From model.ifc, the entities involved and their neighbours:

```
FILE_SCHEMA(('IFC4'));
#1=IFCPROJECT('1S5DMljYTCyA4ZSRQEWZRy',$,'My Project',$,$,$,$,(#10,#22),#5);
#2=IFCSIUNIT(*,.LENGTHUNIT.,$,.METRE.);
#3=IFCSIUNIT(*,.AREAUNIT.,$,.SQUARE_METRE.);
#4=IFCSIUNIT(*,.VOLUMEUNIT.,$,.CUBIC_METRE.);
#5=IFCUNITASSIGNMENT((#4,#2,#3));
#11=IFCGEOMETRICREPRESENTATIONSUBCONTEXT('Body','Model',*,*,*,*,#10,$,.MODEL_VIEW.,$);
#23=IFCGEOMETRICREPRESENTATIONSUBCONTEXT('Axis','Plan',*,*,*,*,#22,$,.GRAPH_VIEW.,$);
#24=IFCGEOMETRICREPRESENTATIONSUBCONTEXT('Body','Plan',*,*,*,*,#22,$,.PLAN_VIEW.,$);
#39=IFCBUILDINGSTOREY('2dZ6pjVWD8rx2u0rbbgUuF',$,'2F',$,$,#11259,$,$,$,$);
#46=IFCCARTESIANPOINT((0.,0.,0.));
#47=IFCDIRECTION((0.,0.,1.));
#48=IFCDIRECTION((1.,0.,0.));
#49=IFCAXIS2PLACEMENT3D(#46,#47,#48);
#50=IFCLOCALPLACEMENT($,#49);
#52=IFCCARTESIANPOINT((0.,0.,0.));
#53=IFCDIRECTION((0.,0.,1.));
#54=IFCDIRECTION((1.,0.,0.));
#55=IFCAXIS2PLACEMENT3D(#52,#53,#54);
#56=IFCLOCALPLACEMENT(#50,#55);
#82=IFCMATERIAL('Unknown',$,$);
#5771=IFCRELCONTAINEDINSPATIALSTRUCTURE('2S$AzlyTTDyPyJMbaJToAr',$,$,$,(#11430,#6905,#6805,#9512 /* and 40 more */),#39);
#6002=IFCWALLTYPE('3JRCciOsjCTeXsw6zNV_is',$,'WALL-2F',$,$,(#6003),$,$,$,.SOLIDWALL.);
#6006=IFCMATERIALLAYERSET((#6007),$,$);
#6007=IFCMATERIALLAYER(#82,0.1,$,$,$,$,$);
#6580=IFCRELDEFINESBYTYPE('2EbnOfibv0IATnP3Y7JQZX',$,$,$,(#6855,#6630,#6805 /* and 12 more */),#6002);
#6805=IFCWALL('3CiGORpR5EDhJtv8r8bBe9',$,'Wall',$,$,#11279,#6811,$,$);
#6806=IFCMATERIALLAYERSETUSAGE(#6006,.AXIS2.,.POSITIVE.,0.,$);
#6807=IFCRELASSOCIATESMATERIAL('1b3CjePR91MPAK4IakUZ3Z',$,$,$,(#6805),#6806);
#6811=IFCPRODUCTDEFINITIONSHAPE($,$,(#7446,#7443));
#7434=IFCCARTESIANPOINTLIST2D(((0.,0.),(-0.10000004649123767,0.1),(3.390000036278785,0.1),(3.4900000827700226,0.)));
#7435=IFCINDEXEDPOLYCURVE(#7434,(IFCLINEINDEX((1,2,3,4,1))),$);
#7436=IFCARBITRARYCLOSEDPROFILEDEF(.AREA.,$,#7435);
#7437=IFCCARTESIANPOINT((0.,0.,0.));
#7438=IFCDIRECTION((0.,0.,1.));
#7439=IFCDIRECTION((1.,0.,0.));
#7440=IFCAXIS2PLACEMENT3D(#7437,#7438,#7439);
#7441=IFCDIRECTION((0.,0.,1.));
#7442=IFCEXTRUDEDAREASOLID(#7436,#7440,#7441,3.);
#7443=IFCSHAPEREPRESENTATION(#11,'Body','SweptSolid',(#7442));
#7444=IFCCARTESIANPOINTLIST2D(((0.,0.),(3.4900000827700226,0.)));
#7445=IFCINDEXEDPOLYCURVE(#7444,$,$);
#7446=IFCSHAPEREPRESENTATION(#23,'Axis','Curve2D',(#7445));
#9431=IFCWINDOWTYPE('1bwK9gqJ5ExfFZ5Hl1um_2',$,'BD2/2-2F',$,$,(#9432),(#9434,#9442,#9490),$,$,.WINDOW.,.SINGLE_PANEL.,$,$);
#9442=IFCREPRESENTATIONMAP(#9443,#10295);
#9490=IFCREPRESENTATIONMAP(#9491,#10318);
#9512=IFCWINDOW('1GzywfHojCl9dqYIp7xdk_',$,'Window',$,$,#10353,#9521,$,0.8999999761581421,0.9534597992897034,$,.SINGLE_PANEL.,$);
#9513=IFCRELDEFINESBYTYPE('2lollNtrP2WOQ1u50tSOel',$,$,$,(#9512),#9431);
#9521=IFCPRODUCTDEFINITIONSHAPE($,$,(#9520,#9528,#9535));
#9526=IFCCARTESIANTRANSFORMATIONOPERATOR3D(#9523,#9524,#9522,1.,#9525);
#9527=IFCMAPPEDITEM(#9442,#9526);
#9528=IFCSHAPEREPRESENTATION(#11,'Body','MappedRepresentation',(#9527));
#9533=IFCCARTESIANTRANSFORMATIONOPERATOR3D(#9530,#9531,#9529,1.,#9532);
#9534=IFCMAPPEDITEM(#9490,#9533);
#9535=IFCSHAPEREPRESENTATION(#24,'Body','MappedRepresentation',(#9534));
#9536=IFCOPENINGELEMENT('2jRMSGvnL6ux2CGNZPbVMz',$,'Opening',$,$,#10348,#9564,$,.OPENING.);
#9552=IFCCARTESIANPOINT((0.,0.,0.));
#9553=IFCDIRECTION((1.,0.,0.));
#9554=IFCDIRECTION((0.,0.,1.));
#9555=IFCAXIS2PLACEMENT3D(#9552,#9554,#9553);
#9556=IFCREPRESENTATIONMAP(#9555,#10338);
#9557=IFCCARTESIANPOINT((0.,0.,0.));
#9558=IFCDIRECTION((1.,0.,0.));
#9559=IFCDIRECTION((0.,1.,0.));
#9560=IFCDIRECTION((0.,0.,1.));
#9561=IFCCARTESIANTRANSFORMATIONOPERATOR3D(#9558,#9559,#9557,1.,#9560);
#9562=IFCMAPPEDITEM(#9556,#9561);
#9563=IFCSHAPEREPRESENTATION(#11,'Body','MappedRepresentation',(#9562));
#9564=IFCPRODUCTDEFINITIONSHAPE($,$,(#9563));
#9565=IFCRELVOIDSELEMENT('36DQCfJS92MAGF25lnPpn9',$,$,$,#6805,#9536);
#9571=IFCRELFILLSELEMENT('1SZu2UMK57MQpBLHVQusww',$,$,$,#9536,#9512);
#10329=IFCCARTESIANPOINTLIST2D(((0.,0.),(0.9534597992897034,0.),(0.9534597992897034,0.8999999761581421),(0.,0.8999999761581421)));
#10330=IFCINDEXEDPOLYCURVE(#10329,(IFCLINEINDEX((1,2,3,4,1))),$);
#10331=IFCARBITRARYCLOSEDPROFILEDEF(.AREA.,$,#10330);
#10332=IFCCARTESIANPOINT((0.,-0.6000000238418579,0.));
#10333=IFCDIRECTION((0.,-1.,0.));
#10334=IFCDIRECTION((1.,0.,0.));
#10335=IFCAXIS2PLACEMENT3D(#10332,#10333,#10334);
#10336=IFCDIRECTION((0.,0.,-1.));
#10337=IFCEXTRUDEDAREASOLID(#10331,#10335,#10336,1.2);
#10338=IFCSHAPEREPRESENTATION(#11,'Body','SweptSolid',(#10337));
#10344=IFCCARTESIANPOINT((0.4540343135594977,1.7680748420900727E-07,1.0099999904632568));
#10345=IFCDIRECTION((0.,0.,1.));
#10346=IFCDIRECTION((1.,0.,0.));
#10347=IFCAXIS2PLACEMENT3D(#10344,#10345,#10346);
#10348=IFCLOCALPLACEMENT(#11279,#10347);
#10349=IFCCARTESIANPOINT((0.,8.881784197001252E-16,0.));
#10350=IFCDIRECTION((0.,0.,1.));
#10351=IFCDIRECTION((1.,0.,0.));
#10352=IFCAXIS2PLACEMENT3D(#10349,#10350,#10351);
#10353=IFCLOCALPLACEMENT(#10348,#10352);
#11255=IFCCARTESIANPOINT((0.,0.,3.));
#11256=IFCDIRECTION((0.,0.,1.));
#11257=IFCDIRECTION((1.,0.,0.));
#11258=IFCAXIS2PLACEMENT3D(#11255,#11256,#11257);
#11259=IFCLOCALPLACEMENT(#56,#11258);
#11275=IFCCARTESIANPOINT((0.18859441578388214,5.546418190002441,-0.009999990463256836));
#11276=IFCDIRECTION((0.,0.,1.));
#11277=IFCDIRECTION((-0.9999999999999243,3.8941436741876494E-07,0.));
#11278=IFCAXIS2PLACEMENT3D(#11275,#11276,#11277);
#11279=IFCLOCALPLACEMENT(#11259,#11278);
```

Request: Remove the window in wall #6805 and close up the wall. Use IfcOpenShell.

```python
import ifcopenshell
import ifcopenshell.api.feature
import ifcopenshell.api.root
import ifcopenshell.geom
import ifcopenshell.util.shape

model = ifcopenshell.open("model.ifc")
settings = ifcopenshell.geom.settings()


def volume(element):
    """Net volume in cubic metres, openings subtracted."""
    shape = ifcopenshell.geom.create_shape(settings, element)
    return ifcopenshell.util.shape.get_volume(shape.geometry)


window = model.by_id(9512)
opening = window.FillsVoids[0].RelatingOpeningElement
wall = opening.VoidsElements[0].RelatingBuildingElement
before = volume(wall)

ifcopenshell.api.root.remove_product(model, product=window)
ifcopenshell.api.feature.remove_feature(model, feature=opening)

after = volume(wall)

print(f"wall volume {before:.3f} -> {after:.3f} m3")

model.write("model_rev.ifc")
```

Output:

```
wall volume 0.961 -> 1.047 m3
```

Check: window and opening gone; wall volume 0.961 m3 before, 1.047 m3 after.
